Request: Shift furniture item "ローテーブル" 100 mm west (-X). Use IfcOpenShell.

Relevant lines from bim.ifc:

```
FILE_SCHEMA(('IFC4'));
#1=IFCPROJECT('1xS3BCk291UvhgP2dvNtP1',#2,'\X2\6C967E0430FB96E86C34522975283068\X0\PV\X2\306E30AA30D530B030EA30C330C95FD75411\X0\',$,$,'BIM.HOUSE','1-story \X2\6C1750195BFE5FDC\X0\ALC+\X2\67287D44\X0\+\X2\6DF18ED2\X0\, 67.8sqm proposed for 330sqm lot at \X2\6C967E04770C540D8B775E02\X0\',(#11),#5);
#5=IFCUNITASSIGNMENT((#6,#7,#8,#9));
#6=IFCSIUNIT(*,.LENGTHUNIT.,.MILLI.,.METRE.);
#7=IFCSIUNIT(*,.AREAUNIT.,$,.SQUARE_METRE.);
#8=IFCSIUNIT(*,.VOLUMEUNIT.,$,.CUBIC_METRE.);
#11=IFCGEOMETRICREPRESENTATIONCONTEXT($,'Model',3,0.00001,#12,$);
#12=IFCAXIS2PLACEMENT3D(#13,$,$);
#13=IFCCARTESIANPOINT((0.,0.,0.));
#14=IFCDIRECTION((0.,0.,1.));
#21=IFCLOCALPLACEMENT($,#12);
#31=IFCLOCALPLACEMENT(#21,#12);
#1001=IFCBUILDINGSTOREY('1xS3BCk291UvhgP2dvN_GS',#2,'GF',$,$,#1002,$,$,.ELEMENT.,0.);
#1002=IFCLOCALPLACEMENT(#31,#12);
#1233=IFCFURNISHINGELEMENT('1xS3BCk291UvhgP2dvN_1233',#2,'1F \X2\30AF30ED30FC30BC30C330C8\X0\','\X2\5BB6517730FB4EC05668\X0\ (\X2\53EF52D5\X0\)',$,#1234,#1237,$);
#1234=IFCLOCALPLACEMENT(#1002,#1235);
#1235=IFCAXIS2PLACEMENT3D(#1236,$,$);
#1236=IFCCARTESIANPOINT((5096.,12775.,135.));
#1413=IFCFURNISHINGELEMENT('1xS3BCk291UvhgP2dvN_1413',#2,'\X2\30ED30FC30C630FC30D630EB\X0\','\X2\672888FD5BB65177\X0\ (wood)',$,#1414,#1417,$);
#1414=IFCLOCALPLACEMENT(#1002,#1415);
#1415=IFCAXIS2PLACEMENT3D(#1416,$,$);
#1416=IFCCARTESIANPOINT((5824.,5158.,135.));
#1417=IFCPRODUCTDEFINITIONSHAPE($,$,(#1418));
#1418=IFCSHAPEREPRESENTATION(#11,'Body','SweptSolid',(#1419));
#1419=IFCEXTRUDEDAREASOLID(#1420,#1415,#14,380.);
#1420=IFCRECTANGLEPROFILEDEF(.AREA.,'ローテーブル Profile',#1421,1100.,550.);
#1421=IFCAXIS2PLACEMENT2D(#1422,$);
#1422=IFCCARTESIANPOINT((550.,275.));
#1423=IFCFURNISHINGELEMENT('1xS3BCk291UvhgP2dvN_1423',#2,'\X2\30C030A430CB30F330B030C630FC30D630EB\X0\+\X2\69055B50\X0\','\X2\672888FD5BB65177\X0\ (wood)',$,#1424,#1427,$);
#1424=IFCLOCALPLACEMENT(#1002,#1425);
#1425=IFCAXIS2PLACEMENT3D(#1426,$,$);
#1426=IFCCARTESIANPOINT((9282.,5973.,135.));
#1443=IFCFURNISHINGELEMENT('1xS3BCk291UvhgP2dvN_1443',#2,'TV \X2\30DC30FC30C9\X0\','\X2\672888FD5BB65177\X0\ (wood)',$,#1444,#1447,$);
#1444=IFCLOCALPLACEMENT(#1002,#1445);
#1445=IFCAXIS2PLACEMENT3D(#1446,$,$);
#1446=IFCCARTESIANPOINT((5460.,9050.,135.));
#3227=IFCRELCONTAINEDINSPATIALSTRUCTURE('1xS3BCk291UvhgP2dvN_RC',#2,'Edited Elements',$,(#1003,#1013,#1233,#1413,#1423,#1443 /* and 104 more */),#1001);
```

```python
import ifcopenshell
import ifcopenshell.api.geometry
import ifcopenshell.util.placement
import ifcopenshell.util.unit

model = ifcopenshell.open("bim.ifc")
unit_scale = ifcopenshell.util.unit.calculate_unit_scale(model)

item = model.by_guid("1xS3BCk291UvhgP2dvN_1413")
matrix = ifcopenshell.util.placement.get_local_placement(item.ObjectPlacement)
matrix[0, 3] -= 0.1 / unit_scale
ifcopenshell.api.geometry.edit_object_placement(model, product=item, matrix=matrix, is_si=False)

print(ifcopenshell.util.placement.get_local_placement(item.ObjectPlacement).round(3) + 0.0)

model.write("bim_edited.ifc")
```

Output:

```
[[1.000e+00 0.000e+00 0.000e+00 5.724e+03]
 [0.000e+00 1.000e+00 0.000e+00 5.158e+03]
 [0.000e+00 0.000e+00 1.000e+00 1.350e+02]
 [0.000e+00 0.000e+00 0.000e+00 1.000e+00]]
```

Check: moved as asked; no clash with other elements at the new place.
